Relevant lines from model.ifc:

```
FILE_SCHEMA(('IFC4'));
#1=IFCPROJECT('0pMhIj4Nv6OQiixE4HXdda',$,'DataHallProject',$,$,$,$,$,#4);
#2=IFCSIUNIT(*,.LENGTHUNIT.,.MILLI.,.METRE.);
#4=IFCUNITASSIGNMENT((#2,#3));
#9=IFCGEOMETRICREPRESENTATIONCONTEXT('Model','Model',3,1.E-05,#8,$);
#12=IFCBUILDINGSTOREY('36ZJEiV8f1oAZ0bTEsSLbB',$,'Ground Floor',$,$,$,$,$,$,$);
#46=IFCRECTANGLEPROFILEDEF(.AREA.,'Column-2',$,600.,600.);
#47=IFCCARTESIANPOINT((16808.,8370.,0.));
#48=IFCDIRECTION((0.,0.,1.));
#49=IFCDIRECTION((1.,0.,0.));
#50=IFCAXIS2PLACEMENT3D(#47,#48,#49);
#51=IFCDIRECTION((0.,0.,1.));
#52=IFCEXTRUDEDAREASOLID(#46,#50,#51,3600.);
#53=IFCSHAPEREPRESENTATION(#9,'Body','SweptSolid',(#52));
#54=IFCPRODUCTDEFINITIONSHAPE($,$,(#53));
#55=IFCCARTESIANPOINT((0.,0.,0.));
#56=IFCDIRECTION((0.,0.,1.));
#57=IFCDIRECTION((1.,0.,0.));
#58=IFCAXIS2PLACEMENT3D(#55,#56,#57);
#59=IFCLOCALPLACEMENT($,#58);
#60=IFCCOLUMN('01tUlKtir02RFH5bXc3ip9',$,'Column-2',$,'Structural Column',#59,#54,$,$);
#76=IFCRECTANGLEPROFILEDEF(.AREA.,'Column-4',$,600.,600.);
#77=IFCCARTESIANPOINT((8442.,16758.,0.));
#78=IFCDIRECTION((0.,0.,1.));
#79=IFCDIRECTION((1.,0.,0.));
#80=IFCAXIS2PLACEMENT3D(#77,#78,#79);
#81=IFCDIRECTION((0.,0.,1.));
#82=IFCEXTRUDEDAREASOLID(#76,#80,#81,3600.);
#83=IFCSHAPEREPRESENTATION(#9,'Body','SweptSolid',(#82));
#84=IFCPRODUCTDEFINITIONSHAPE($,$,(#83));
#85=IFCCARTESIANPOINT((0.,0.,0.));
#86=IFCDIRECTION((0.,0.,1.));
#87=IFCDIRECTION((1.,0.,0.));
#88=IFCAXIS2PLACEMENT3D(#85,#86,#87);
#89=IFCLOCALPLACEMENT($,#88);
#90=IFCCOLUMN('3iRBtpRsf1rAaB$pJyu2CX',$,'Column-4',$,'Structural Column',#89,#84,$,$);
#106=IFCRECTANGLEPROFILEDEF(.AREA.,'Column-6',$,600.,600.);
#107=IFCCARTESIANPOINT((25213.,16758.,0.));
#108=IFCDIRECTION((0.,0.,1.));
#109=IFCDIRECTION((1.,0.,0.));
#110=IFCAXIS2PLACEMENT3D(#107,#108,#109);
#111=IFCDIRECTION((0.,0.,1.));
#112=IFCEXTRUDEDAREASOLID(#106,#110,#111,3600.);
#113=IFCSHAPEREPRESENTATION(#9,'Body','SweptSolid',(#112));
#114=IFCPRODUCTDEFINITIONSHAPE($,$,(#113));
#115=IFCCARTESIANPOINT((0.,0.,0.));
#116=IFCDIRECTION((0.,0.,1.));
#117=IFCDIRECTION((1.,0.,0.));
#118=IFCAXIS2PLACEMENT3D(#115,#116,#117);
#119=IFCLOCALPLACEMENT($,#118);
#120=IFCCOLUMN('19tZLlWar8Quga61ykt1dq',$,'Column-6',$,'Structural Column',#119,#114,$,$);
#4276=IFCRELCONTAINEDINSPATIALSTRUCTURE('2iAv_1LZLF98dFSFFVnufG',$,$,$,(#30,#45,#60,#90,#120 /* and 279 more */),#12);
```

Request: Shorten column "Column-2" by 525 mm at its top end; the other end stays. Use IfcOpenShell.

```python
import ifcopenshell
import ifcopenshell.util.unit

model = ifcopenshell.open("model.ifc")
unit_scale = ifcopenshell.util.unit.calculate_unit_scale(model)

member = model.by_guid("01tUlKtir02RFH5bXc3ip9")
change = -0.525 / unit_scale

# The extrusion runs towards the end named, so only its depth changes.
body = next(r for r in member.Representation.Representations if r.RepresentationIdentifier == "Body")
solid = body.Items[0]
old_length = solid.Depth
solid.Depth += change

print(f"length {old_length:g} -> {solid.Depth:g}")

model.write("model_rev.ifc")
```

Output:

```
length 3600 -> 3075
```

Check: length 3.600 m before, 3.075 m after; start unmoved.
